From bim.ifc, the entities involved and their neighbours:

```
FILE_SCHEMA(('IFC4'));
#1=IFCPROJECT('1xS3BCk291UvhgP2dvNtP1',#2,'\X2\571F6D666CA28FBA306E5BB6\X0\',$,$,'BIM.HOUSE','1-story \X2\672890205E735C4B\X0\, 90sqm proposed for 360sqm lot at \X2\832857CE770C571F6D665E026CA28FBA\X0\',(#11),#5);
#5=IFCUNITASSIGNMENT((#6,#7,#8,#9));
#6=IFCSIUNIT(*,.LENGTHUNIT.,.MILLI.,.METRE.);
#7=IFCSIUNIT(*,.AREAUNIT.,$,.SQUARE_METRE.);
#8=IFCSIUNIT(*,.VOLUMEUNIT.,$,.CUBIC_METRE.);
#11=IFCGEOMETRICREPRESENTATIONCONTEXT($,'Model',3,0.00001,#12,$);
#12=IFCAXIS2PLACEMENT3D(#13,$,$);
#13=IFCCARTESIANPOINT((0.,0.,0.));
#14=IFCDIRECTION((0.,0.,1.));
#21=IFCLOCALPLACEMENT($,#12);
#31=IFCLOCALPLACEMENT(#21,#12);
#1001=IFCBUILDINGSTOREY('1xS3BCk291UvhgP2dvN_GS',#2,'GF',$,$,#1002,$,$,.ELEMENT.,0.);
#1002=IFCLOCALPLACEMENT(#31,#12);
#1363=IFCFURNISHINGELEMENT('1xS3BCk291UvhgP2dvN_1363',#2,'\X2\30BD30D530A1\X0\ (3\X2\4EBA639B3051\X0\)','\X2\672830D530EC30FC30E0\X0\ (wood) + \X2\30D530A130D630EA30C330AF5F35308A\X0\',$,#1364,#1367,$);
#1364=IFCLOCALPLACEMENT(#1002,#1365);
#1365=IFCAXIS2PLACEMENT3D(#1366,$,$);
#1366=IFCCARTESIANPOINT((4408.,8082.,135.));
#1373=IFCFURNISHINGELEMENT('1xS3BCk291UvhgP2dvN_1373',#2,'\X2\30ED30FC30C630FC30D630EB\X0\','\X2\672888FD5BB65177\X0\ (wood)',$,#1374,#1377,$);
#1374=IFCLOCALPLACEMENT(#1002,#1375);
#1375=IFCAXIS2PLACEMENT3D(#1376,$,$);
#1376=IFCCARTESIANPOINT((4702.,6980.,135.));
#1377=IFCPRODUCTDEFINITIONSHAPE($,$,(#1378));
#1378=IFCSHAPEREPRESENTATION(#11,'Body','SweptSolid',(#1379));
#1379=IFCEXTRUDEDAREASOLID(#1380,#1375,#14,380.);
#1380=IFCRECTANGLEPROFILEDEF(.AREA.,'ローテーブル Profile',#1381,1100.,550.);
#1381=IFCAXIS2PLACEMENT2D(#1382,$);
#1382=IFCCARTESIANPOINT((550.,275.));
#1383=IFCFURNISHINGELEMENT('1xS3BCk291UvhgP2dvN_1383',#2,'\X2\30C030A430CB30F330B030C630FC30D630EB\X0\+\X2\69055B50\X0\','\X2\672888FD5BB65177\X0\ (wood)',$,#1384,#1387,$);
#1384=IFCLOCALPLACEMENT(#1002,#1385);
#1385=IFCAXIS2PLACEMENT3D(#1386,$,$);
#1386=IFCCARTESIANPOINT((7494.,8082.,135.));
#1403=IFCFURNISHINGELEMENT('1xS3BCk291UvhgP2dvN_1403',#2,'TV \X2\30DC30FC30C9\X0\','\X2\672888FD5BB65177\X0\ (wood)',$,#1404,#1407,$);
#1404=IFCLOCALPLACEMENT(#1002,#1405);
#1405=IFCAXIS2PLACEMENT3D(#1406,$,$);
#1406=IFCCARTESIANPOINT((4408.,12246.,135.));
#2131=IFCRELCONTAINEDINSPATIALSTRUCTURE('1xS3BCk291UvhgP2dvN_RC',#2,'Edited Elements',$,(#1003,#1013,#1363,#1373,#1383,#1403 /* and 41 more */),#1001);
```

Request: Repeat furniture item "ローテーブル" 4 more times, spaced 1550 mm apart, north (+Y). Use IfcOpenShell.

```python
import numpy as np
import ifcopenshell
import ifcopenshell.api.geometry
import ifcopenshell.api.root
import ifcopenshell.util.element
import ifcopenshell.util.placement
import ifcopenshell.util.unit

model = ifcopenshell.open("bim.ifc")
unit_scale = ifcopenshell.util.unit.calculate_unit_scale(model)


def reuse_history(source, copy):
    """copy_class also copies each property set's owner history, people and application; keep the originals."""
    for rel in copy.IsDefinedBy:
        if rel.is_a("IfcRelDefinesByProperties") and (history := rel.RelatingPropertyDefinition.OwnerHistory):
            rel.RelatingPropertyDefinition.OwnerHistory = source.OwnerHistory
            ifcopenshell.util.element.remove_deep2(model, history)


source = model.by_guid("1xS3BCk291UvhgP2dvN_1373")
base = ifcopenshell.util.placement.get_local_placement(source.ObjectPlacement)
step = np.array([0.0, 1.0, 0.0]) * 1.55 / unit_scale

for i in range(1, 5):
    copy = ifcopenshell.api.root.copy_class(model, product=source)
    copy.Representation = ifcopenshell.util.element.copy_deep(
        model, source.Representation, exclude=["IfcGeometricRepresentationContext", "IfcRepresentationMap"]
    )
    reuse_history(source, copy)
    matrix = base.copy()
    matrix[:3, 3] += i * step
    print("added at", matrix[:3, 3].round(3) + 0.0)
    ifcopenshell.api.geometry.edit_object_placement(model, product=copy, matrix=matrix, is_si=False)

model.write("bim_edited.ifc")
```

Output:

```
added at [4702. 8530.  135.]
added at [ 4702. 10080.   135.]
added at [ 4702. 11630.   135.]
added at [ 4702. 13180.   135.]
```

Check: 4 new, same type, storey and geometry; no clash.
